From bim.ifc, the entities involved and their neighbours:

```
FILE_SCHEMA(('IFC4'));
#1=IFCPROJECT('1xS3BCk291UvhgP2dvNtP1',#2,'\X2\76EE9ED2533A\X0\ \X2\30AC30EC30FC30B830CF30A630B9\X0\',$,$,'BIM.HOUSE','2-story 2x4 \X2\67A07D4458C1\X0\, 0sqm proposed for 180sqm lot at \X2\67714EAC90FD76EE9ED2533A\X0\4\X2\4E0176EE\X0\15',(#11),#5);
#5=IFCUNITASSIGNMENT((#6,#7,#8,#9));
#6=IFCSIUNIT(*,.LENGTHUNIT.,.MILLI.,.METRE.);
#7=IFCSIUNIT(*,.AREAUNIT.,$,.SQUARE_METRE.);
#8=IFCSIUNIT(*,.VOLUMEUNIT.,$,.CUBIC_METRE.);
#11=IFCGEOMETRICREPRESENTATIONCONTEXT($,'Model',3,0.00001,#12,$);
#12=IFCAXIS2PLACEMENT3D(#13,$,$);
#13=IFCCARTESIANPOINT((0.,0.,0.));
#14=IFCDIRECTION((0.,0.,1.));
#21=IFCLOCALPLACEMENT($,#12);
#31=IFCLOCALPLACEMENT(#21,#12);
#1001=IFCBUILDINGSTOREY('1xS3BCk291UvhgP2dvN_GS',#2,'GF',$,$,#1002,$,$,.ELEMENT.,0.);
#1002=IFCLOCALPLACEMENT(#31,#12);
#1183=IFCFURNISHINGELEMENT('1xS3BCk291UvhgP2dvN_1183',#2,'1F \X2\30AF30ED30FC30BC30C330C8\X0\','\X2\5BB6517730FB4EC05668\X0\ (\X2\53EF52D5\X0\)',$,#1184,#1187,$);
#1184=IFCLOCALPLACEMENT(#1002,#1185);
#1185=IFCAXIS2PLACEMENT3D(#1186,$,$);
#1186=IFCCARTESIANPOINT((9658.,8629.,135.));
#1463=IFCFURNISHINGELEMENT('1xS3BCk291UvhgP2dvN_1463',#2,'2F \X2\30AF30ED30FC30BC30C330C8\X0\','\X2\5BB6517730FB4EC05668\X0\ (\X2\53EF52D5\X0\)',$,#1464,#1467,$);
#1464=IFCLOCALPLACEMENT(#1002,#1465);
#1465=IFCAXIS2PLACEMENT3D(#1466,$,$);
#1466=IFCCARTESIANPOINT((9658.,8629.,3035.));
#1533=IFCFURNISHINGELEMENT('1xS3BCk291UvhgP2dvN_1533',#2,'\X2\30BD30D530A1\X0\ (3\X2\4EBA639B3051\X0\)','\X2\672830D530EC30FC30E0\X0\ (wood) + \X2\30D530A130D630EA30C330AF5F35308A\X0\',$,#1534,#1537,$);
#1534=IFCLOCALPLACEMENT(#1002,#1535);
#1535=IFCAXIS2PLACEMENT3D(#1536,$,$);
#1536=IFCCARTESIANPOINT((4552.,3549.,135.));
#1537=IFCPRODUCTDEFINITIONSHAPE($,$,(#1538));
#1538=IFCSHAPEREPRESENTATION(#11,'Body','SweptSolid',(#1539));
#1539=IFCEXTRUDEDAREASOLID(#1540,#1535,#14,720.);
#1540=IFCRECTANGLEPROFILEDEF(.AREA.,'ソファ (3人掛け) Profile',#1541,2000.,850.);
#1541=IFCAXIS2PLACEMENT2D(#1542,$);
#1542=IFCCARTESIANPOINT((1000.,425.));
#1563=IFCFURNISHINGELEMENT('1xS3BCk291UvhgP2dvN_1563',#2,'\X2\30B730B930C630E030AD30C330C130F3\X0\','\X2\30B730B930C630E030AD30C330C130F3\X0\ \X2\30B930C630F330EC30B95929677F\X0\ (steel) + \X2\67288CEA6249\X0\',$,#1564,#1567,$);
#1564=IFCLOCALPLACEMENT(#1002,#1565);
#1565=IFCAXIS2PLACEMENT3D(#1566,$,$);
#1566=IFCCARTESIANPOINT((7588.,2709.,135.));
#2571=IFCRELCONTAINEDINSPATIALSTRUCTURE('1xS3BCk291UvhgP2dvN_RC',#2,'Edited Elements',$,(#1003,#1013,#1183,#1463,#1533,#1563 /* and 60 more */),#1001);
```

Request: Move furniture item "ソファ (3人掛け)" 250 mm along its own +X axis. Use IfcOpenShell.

```python
import ifcopenshell
import ifcopenshell.api.geometry
import ifcopenshell.util.placement

model = ifcopenshell.open("bim.ifc")

item = model.by_guid("1xS3BCk291UvhgP2dvN_1533")
matrix = ifcopenshell.util.placement.get_local_placement(item.ObjectPlacement)
matrix[:3, 3] += matrix[:3, 0] * 250.0
ifcopenshell.api.geometry.edit_object_placement(model, product=item, matrix=matrix, is_si=False)

print(ifcopenshell.util.placement.get_local_placement(item.ObjectPlacement).round(3) + 0.0)

model.write("bim-out.ifc")
```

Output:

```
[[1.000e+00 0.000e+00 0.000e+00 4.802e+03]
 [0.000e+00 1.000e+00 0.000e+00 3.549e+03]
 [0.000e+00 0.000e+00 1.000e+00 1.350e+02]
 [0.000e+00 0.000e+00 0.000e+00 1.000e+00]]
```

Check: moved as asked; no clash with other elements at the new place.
